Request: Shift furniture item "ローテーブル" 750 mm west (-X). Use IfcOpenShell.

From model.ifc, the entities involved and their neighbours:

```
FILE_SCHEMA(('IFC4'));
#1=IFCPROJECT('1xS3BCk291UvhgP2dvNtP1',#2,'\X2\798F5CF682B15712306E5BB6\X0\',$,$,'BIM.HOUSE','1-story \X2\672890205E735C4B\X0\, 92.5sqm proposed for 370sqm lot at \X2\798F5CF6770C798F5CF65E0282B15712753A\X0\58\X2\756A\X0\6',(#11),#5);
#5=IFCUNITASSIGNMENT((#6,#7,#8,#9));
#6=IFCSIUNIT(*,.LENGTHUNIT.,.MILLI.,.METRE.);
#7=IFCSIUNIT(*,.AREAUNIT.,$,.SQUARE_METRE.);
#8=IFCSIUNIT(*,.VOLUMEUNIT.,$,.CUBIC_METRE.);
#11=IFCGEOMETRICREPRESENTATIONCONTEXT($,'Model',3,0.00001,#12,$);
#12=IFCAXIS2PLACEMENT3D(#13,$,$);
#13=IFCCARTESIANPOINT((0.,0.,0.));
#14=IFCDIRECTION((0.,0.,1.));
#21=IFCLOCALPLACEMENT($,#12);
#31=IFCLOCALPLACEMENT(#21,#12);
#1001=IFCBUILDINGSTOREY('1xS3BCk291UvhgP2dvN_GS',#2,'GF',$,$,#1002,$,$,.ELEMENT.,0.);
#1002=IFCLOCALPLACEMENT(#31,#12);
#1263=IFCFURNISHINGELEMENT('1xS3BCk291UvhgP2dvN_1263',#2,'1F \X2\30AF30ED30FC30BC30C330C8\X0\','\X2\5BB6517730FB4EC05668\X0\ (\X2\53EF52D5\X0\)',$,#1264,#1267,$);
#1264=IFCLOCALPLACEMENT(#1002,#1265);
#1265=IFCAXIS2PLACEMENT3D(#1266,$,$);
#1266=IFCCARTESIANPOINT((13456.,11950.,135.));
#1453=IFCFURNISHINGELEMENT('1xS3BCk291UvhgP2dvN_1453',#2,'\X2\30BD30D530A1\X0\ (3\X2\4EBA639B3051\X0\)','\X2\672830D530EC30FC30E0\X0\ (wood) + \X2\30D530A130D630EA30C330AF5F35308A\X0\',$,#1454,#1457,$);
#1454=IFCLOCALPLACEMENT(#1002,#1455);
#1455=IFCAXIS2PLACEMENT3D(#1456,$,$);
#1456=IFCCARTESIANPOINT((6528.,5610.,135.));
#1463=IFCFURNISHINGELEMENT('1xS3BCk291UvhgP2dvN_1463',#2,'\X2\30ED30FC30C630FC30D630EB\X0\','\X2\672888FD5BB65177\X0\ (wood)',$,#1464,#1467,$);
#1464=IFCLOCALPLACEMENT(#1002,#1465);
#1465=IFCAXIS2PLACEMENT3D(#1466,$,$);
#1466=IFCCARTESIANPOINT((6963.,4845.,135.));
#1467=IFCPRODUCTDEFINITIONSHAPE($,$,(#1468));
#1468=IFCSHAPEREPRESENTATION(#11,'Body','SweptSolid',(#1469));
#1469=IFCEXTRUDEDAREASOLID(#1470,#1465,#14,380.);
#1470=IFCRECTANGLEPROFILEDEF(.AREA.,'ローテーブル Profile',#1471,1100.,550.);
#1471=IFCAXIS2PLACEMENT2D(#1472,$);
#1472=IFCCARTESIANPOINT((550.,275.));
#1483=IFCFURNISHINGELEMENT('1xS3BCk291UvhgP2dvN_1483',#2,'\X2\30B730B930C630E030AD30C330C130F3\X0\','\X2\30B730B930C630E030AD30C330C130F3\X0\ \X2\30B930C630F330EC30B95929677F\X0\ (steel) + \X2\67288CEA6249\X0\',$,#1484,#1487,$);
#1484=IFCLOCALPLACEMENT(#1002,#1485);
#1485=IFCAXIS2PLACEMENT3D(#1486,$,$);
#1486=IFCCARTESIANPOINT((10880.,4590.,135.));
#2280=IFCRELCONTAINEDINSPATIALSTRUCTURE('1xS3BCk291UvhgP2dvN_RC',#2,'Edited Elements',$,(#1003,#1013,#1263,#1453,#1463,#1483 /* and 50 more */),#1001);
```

```python
import ifcopenshell
import ifcopenshell.api.geometry
import ifcopenshell.util.placement

model = ifcopenshell.open("model.ifc")

item = model.by_guid("1xS3BCk291UvhgP2dvN_1463")
matrix = ifcopenshell.util.placement.get_local_placement(item.ObjectPlacement)
matrix[0, 3] -= 750.0
ifcopenshell.api.geometry.edit_object_placement(model, product=item, matrix=matrix, is_si=False)

print(ifcopenshell.util.placement.get_local_placement(item.ObjectPlacement).round(3) + 0.0)

model.write("model_updated.ifc")
```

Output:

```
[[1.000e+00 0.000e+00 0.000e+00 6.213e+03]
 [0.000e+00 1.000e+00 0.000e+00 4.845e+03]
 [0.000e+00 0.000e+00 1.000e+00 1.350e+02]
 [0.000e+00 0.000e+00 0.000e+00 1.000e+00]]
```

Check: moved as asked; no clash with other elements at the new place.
